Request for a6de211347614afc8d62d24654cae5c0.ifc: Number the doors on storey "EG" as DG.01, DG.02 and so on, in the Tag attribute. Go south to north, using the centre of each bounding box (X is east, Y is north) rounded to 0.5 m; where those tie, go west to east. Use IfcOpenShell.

First a look at what the model holds.

```python
import ifcopenshell
import ifcopenshell.util.element
import ifcopenshell.util.placement

model = ifcopenshell.open("a6de211347614afc8d62d24654cae5c0.ifc")
print(model.schema)
storey = next(s for s in model.by_type("IfcBuildingStorey") if s.Name == "EG")
doors = [e for e in ifcopenshell.util.element.get_decomposition(storey) if e.is_a("IfcDoor")]
for e in sorted(doors, key=lambda e: e.id()):
    origin = ifcopenshell.util.placement.get_local_placement(e.ObjectPlacement)[:3, 3]
    print(e.id(), e.Tag, e.Name, origin.round(2) + 0.0, sep=" | ")
```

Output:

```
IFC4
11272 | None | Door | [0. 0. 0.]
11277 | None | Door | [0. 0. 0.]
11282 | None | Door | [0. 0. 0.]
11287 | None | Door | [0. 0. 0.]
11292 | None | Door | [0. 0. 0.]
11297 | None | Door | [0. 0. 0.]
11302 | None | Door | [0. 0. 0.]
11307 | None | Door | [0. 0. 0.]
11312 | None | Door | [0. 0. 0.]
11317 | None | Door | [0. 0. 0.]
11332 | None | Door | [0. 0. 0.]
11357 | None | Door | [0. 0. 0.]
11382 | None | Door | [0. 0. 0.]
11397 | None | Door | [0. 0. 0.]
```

```python
import ifcopenshell
import ifcopenshell.geom
import ifcopenshell.util.element
import ifcopenshell.util.shape

model = ifcopenshell.open("a6de211347614afc8d62d24654cae5c0.ifc")
settings = ifcopenshell.geom.settings()
settings.set("use-world-coords", True)


def centre(element):
    shape = ifcopenshell.geom.create_shape(settings, element)
    return ifcopenshell.util.shape.get_bbox_centroid(shape.geometry)


storey = next(s for s in model.by_type("IfcBuildingStorey") if s.Name == "EG")
doors = [e for e in ifcopenshell.util.element.get_decomposition(storey) if e.is_a("IfcDoor")]

# Insertion points can sit at a corner or the storey origin, so sort by the geometry (in metres).
centres = {e: centre(e) for e in doors}
doors.sort(key=lambda e: (round(centres[e][1] / 0.5), centres[e][0]))

for i, e in enumerate(doors, start=1):
    number = f"DG.{i:02d}"
    e.Tag = number
    print(e.id(), number)

model.write("a6de211347614afc8d62d24654cae5c0-out.ifc")
```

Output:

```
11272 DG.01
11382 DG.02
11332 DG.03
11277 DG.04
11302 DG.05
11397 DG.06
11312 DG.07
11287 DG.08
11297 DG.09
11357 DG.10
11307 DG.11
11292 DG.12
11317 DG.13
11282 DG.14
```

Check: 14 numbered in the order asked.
